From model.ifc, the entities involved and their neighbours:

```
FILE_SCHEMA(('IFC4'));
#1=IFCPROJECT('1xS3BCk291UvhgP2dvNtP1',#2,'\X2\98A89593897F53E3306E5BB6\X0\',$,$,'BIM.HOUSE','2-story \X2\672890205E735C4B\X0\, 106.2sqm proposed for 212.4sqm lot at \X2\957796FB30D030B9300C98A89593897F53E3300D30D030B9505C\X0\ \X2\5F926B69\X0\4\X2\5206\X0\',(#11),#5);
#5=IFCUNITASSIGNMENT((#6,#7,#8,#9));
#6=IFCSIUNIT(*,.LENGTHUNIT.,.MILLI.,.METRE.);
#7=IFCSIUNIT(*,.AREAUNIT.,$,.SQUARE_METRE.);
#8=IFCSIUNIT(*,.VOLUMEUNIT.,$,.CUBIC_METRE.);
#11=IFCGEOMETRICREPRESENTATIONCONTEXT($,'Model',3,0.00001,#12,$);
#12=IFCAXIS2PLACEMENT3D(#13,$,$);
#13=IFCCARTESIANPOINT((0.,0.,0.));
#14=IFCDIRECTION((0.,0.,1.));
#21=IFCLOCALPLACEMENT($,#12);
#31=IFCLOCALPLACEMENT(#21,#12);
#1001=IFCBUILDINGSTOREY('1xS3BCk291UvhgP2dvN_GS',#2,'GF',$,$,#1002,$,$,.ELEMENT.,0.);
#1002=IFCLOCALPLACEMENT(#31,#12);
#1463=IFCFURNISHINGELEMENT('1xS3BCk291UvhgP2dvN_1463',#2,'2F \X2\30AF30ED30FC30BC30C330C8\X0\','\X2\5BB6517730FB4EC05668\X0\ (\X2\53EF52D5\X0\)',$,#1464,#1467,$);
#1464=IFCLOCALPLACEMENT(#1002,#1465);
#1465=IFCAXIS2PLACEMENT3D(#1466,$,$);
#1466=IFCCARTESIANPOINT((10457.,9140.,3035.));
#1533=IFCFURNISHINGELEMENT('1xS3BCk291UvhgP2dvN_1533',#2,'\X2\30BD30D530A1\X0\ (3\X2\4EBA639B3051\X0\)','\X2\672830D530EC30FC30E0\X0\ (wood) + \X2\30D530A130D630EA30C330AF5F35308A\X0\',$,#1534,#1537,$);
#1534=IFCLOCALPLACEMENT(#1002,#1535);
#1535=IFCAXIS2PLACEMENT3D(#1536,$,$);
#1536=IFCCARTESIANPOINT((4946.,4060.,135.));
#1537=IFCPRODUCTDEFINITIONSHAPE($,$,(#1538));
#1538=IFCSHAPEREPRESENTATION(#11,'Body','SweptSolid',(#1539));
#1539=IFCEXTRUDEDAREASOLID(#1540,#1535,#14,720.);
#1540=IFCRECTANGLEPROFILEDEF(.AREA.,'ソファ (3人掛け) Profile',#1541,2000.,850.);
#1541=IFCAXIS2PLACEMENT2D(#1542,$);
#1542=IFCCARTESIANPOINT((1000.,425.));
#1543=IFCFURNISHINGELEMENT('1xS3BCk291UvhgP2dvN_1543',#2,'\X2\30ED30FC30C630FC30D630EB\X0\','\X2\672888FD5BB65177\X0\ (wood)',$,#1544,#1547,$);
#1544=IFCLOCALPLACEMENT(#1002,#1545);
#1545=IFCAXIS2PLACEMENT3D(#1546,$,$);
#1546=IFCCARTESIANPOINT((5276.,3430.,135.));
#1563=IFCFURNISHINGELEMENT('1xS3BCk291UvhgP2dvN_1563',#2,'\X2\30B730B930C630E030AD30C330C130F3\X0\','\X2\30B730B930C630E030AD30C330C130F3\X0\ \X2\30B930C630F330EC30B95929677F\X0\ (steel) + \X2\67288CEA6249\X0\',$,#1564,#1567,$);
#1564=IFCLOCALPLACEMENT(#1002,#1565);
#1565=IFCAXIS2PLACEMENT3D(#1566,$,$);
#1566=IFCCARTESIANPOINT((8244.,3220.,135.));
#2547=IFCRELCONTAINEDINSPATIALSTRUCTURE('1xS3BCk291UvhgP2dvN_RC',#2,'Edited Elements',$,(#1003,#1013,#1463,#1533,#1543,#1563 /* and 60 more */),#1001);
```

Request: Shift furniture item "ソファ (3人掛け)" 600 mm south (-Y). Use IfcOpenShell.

```python
import ifcopenshell
import ifcopenshell.api.geometry
import ifcopenshell.util.placement

model = ifcopenshell.open("model.ifc")

item = model.by_guid("1xS3BCk291UvhgP2dvN_1533")
matrix = ifcopenshell.util.placement.get_local_placement(item.ObjectPlacement)
matrix[1, 3] -= 600.0
ifcopenshell.api.geometry.edit_object_placement(model, product=item, matrix=matrix, is_si=False)

print(ifcopenshell.util.placement.get_local_placement(item.ObjectPlacement).round(3) + 0.0)

model.write("model-out.ifc")
```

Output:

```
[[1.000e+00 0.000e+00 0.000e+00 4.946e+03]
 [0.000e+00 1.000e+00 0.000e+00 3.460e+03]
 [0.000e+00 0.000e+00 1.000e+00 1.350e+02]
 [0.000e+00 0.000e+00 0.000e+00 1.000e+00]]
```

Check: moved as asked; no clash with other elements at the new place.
